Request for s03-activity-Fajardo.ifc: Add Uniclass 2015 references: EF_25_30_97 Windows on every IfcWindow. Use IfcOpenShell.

First a look at what the model holds.

```python
import ifcopenshell

model = ifcopenshell.open("s03-activity-Fajardo.ifc")
print(model.schema)
print("classifications:", [c.Name for c in model.by_type("IfcClassification")])
for ifc_class in ("IfcDoor", "IfcRoof", "IfcStair", "IfcWall", "IfcWindow"):
    print(ifc_class, len(model.by_type(ifc_class)))
```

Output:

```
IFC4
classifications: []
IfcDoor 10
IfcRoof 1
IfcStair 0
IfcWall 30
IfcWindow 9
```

```python
import ifcopenshell
import ifcopenshell.api.classification

model = ifcopenshell.open("s03-activity-Fajardo.ifc")

system = ifcopenshell.api.classification.add_classification(model, classification="Uniclass 2015")

codes = {
    "IfcWindow": ("EF_25_30_97", "Windows"),
}
for ifc_class, (code, name) in codes.items():
    products = model.by_type(ifc_class)
    ifcopenshell.api.classification.add_reference(
        model, products=products, classification=system, identification=code, name=name
    )
    print(code, len(products))

model.write("s03-activity-Fajardo_rev.ifc")
```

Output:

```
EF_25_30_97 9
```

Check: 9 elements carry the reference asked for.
